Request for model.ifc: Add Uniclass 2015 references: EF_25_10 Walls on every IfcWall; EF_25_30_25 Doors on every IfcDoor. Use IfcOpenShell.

First a look at what the model holds.

```python
import ifcopenshell

model = ifcopenshell.open("model.ifc")
print(model.schema)
print("classifications:", [c.Name for c in model.by_type("IfcClassification")])
for ifc_class in ("IfcDoor", "IfcRoof", "IfcStair", "IfcWall", "IfcWindow"):
    print(ifc_class, len(model.by_type(ifc_class)))
```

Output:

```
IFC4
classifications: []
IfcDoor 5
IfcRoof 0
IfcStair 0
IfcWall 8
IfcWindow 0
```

```python
import ifcopenshell
import ifcopenshell.api.classification

model = ifcopenshell.open("model.ifc")

system = ifcopenshell.api.classification.add_classification(model, classification="Uniclass 2015")

codes = {
    "IfcWall": ("EF_25_10", "Walls"),
    "IfcDoor": ("EF_25_30_25", "Doors"),
}
for ifc_class, (code, name) in codes.items():
    products = model.by_type(ifc_class)
    ifcopenshell.api.classification.add_reference(
        model, products=products, classification=system, identification=code, name=name
    )
    print(code, len(products))

model.write("model_edited.ifc")
```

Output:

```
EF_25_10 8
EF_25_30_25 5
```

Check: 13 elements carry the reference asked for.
